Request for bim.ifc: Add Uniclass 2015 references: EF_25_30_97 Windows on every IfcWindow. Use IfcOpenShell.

First a look at what the model holds.

```python
import ifcopenshell

model = ifcopenshell.open("bim.ifc")
print(model.schema)
print("classifications:", [c.Name for c in model.by_type("IfcClassification")])
for ifc_class in ("IfcDoor", "IfcRoof", "IfcStair", "IfcWall", "IfcWindow"):
    print(ifc_class, len(model.by_type(ifc_class)))
```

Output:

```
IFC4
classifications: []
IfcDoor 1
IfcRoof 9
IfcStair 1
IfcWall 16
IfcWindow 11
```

```python
import ifcopenshell
import ifcopenshell.api.classification

model = ifcopenshell.open("bim.ifc")

system = ifcopenshell.api.classification.add_classification(model, classification="Uniclass 2015")

codes = {
    "IfcWindow": ("EF_25_30_97", "Windows"),
}
for ifc_class, (code, name) in codes.items():
    products = model.by_type(ifc_class)
    ifcopenshell.api.classification.add_reference(
        model, products=products, classification=system, identification=code, name=name
    )
    print(code, len(products))

model.write("bim_v2.ifc")
```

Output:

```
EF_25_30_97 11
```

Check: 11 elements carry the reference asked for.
